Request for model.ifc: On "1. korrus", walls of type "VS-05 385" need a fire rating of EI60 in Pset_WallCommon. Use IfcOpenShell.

First a look at what the model holds.

```python
import ifcopenshell
import ifcopenshell.util.element

model = ifcopenshell.open("model.ifc")
print(model.schema)
storey = next(s for s in model.by_type("IfcBuildingStorey") if s.Name == "1. korrus")
walls = [e for e in ifcopenshell.util.element.get_decomposition(storey) if e.is_a("IfcWall")]
seen = {}
for e in walls:
    element_type = ifcopenshell.util.element.get_type(e)
    key = (element_type.Name if element_type != e and element_type else None, ifcopenshell.util.element.get_pset(e, "Pset_WallCommon", "FireRating"))
    seen[key] = seen.get(key, 0) + 1
for (name, value), count in sorted(seen.items(), key=str):
    print(count, "x", name, "|", value)
```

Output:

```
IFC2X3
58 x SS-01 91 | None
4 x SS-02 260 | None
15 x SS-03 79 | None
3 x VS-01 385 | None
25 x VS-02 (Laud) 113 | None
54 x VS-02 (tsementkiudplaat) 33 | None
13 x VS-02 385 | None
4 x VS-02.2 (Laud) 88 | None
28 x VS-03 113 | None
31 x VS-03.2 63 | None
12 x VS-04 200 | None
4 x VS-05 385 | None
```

```python
import ifcopenshell
import ifcopenshell.api.pset
import ifcopenshell.util.element

model = ifcopenshell.open("model.ifc")

storey = next(s for s in model.by_type("IfcBuildingStorey") if s.Name == "1. korrus")
walls = [e for e in ifcopenshell.util.element.get_decomposition(storey) if e.is_a("IfcWall")]

count = 0
for e in walls:
    element_type = ifcopenshell.util.element.get_type(e)
    if element_type in (None, e) or element_type.Name != "VS-05 385":
        continue
    # add_pset returns the element's existing set when there is one.
    pset = ifcopenshell.api.pset.add_pset(model, product=e, name="Pset_WallCommon")
    ifcopenshell.api.pset.edit_pset(model, pset=pset, properties={"FireRating": "EI60"})
    count += 1

print(count, "walls updated")

model.write("model-out.ifc")
```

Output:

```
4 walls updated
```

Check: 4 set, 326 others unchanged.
